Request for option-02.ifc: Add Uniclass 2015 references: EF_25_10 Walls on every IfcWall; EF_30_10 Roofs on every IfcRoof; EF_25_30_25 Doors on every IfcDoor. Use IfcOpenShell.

First a look at what the model holds.

```python
import ifcopenshell

model = ifcopenshell.open("option-02.ifc")
print(model.schema)
print("classifications:", [c.Name for c in model.by_type("IfcClassification")])
for ifc_class in ("IfcDoor", "IfcRoof", "IfcStair", "IfcWall", "IfcWindow"):
    print(ifc_class, len(model.by_type(ifc_class)))
```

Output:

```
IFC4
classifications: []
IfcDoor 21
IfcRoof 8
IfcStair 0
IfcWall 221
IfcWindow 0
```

```python
import ifcopenshell
import ifcopenshell.api.classification

model = ifcopenshell.open("option-02.ifc")

system = ifcopenshell.api.classification.add_classification(model, classification="Uniclass 2015")

codes = {
    "IfcWall": ("EF_25_10", "Walls"),
    "IfcRoof": ("EF_30_10", "Roofs"),
    "IfcDoor": ("EF_25_30_25", "Doors"),
}
for ifc_class, (code, name) in codes.items():
    products = model.by_type(ifc_class)
    ifcopenshell.api.classification.add_reference(
        model, products=products, classification=system, identification=code, name=name
    )
    print(code, len(products))

model.write("option-02_updated.ifc")
```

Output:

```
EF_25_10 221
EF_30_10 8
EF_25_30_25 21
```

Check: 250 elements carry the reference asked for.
